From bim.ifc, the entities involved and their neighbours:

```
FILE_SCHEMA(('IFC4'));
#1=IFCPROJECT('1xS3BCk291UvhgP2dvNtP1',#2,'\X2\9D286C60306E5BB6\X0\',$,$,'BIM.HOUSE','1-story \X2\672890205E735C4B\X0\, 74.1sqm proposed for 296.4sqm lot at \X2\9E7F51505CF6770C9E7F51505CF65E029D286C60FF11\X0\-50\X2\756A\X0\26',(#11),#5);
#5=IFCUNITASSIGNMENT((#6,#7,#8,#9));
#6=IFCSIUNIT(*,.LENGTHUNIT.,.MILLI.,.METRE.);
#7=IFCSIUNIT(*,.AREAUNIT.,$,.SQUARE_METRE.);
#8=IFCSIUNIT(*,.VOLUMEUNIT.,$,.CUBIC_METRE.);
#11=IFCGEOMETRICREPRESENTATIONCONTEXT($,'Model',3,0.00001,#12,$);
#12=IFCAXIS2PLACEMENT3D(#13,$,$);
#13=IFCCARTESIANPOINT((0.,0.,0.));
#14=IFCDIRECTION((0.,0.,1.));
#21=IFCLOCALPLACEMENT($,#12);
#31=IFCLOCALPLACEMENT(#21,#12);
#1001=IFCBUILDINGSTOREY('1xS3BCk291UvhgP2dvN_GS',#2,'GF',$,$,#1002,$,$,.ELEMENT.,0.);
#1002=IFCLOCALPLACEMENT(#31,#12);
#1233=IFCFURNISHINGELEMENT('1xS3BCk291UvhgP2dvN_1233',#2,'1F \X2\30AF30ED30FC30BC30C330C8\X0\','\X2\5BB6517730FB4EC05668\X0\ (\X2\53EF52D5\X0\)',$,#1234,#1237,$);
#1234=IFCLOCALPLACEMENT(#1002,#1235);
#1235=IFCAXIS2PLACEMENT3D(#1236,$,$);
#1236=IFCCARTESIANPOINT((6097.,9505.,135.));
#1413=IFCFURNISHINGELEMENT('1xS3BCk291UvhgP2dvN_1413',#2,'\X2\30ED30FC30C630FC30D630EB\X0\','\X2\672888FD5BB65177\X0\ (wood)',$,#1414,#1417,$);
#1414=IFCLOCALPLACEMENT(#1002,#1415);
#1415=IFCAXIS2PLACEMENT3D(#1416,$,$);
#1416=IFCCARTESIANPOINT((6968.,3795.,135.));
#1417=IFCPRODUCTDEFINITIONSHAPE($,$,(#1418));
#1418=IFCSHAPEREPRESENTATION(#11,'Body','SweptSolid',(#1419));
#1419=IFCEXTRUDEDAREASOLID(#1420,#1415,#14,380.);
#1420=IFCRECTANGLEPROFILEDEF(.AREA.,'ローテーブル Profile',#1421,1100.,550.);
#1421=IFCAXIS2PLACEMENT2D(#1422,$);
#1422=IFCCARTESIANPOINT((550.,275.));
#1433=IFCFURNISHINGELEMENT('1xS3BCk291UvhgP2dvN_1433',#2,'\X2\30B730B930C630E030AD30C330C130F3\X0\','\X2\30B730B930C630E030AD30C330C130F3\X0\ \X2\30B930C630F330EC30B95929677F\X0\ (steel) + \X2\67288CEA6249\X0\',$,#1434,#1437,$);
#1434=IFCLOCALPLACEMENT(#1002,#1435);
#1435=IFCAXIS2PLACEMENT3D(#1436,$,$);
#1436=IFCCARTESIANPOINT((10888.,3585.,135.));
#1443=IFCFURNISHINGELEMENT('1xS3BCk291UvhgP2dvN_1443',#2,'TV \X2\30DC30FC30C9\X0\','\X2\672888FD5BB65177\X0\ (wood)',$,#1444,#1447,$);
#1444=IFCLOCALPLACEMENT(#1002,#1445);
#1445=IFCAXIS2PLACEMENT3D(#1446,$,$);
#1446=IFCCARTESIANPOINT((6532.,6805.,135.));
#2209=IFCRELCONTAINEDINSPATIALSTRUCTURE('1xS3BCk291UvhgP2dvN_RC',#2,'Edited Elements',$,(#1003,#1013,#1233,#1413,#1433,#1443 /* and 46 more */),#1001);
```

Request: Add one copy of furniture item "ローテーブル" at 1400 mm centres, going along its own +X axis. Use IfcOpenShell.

```python
import ifcopenshell
import ifcopenshell.api.geometry
import ifcopenshell.api.root
import ifcopenshell.util.element
import ifcopenshell.util.placement

model = ifcopenshell.open("bim.ifc")


def reuse_history(source, copy):
    """copy_class also copies each property set's owner history, people and application; keep the originals."""
    for rel in copy.IsDefinedBy:
        if rel.is_a("IfcRelDefinesByProperties") and (history := rel.RelatingPropertyDefinition.OwnerHistory):
            rel.RelatingPropertyDefinition.OwnerHistory = source.OwnerHistory
            ifcopenshell.util.element.remove_deep2(model, history)


source = model.by_guid("1xS3BCk291UvhgP2dvN_1413")
base = ifcopenshell.util.placement.get_local_placement(source.ObjectPlacement)
step = base[:3, 0] * 1400.0

for i in range(1, 2):
    copy = ifcopenshell.api.root.copy_class(model, product=source)
    copy.Representation = ifcopenshell.util.element.copy_deep(
        model, source.Representation, exclude=["IfcGeometricRepresentationContext", "IfcRepresentationMap"]
    )
    reuse_history(source, copy)
    matrix = base.copy()
    matrix[:3, 3] += i * step
    print("added at", matrix[:3, 3].round(3) + 0.0)
    ifcopenshell.api.geometry.edit_object_placement(model, product=copy, matrix=matrix, is_si=False)

model.write("bim-out.ifc")
```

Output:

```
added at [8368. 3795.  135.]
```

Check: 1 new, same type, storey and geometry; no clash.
